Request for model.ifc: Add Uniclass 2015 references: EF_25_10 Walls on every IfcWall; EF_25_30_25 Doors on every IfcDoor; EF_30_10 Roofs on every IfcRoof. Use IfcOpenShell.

First a look at what the model holds.

```python
import ifcopenshell

model = ifcopenshell.open("model.ifc")
print(model.schema)
print("classifications:", [c.Name for c in model.by_type("IfcClassification")])
for ifc_class in ("IfcDoor", "IfcRoof", "IfcStair", "IfcWall", "IfcWindow"):
    print(ifc_class, len(model.by_type(ifc_class)))
```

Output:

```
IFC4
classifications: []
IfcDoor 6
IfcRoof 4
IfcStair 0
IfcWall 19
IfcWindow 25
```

```python
import ifcopenshell
import ifcopenshell.api.classification

model = ifcopenshell.open("model.ifc")

system = ifcopenshell.api.classification.add_classification(model, classification="Uniclass 2015")

codes = {
    "IfcWall": ("EF_25_10", "Walls"),
    "IfcDoor": ("EF_25_30_25", "Doors"),
    "IfcRoof": ("EF_30_10", "Roofs"),
}
for ifc_class, (code, name) in codes.items():
    products = model.by_type(ifc_class)
    ifcopenshell.api.classification.add_reference(
        model, products=products, classification=system, identification=code, name=name
    )
    print(code, len(products))

model.write("model-out.ifc")
```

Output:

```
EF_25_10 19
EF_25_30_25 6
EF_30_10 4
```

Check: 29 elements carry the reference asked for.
